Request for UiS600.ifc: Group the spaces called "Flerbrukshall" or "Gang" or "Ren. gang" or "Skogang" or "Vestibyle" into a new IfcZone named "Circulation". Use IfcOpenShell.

First a look at what the model holds.

```python
import ifcopenshell

model = ifcopenshell.open("UiS600.ifc")
print(model.schema)
seen = {}
for space in model.by_type("IfcSpace"):
    seen[space.LongName] = seen.get(space.LongName, 0) + 1
for name, count in sorted(seen.items(), key=str):
    print(count, "x", name)
print("zones:", [z.Name for z in model.by_type("IfcZone")][:20])
```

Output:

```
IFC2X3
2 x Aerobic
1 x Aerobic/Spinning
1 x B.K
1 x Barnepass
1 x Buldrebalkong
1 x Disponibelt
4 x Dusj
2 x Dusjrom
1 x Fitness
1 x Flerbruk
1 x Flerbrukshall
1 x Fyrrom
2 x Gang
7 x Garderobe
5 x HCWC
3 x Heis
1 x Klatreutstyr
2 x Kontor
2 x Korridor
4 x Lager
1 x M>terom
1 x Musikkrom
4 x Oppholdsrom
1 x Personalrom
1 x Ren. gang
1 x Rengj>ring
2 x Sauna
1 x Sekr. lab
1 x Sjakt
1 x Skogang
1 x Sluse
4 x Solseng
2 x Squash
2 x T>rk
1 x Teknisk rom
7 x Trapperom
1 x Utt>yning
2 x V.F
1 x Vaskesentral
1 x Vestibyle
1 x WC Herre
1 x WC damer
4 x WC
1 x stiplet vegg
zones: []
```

```python
import ifcopenshell
import ifcopenshell.api.group
import ifcopenshell.api.root

model = ifcopenshell.open("UiS600.ifc")

names = {"Flerbrukshall", "Gang", "Ren. gang", "Skogang", "Vestibyle"}
spaces = [s for s in model.by_type("IfcSpace") if s.LongName in names]

zone = ifcopenshell.api.root.create_entity(model, ifc_class="IfcZone", name="Circulation")
ifcopenshell.api.group.assign_group(model, products=spaces, group=zone)
print(len(spaces), "spaces in", zone.Name)

model.write("UiS600_edited.ifc")
```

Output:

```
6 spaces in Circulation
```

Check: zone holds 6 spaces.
